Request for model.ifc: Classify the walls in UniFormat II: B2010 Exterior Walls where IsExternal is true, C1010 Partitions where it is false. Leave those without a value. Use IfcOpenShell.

First a look at what the model holds.

```python
import ifcopenshell
import ifcopenshell.util.element

model = ifcopenshell.open("model.ifc")
print(model.schema)
print("classifications:", [c.Name for c in model.by_type("IfcClassification")])
values = [ifcopenshell.util.element.get_pset(e, "Pset_WallCommon", "IsExternal") for e in model.by_type("IfcWall")]
for value in (True, False, None):
    print("IsExternal", value, values.count(value))
```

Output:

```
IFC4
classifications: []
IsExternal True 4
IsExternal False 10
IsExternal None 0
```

```python
import ifcopenshell
import ifcopenshell.api.classification
import ifcopenshell.util.element

model = ifcopenshell.open("model.ifc")

system = ifcopenshell.api.classification.add_classification(model, classification="UniFormat II")

walls = model.by_type("IfcWall")
external = {e: ifcopenshell.util.element.get_pset(e, "Pset_WallCommon", "IsExternal") for e in walls}
for flag, code, name in ((True, "B2010", "Exterior Walls"), (False, "C1010", "Partitions")):
    products = [e for e in walls if external[e] is flag]
    ifcopenshell.api.classification.add_reference(
        model, products=products, classification=system, identification=code, name=name
    )
    print(code, len(products))

model.write("model_updated.ifc")
```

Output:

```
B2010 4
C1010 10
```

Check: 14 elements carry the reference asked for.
